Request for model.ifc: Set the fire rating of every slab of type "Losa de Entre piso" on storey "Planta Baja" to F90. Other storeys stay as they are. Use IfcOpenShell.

First a look at what the model holds.

```python
import ifcopenshell
import ifcopenshell.util.element

model = ifcopenshell.open("model.ifc")
print(model.schema)
storey = next(s for s in model.by_type("IfcBuildingStorey") if s.Name == "Planta Baja")
slabs = [e for e in ifcopenshell.util.element.get_decomposition(storey) if e.is_a("IfcSlab")]
seen = {}
for e in slabs:
    element_type = ifcopenshell.util.element.get_type(e)
    key = (element_type.Name if element_type != e and element_type else None, ifcopenshell.util.element.get_pset(e, "Pset_SlabCommon", "FireRating"))
    seen[key] = seen.get(key, 0) + 1
for (name, value), count in sorted(seen.items(), key=str):
    print(count, "x", name, "|", value)
```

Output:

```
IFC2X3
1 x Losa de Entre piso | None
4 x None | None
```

```python
import ifcopenshell
import ifcopenshell.api.pset
import ifcopenshell.util.element

model = ifcopenshell.open("model.ifc")

storey = next(s for s in model.by_type("IfcBuildingStorey") if s.Name == "Planta Baja")
slabs = [e for e in ifcopenshell.util.element.get_decomposition(storey) if e.is_a("IfcSlab")]

count = 0
for e in slabs:
    element_type = ifcopenshell.util.element.get_type(e)
    if element_type in (None, e) or element_type.Name != "Losa de Entre piso":
        continue
    # add_pset returns the element's existing set when there is one.
    pset = ifcopenshell.api.pset.add_pset(model, product=e, name="Pset_SlabCommon")
    ifcopenshell.api.pset.edit_pset(model, pset=pset, properties={"FireRating": "F90"})
    count += 1

print(count, "slabs updated")

model.write("model-out.ifc")
```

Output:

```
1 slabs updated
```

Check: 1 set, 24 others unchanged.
